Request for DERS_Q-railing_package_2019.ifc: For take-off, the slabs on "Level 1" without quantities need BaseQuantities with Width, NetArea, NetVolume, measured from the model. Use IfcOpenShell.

First a look at what the model holds.

```python
import ifcopenshell
import ifcopenshell.util.element
import ifcopenshell.util.unit

model = ifcopenshell.open("DERS_Q-railing_package_2019.ifc")
print(model.schema)
for unit_type in ("LENGTHUNIT", "AREAUNIT", "VOLUMEUNIT"):
    print(unit_type, ifcopenshell.util.unit.calculate_unit_scale(model, unit_type))
storey = next(s for s in model.by_type("IfcBuildingStorey") if s.Name == "Level 1")
slabs = [e for e in ifcopenshell.util.element.get_decomposition(storey) if e.is_a("IfcSlab")]
for e in sorted(slabs, key=lambda e: e.id()):
    print(e.id(), e.is_a(), e.Name, list(ifcopenshell.util.element.get_psets(e, qtos_only=True)), sep=" | ")
```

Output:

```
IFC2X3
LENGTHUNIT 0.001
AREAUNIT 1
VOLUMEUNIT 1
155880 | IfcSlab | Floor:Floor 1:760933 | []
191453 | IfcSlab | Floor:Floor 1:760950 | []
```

```python
import ifcopenshell
import ifcopenshell.api.pset
import ifcopenshell.geom
import ifcopenshell.util.element
import ifcopenshell.util.shape
import ifcopenshell.util.unit

model = ifcopenshell.open("DERS_Q-railing_package_2019.ifc")
unit_scale = ifcopenshell.util.unit.calculate_unit_scale(model)
area_scale = ifcopenshell.util.unit.calculate_unit_scale(model, "AREAUNIT")
volume_scale = ifcopenshell.util.unit.calculate_unit_scale(model, "VOLUMEUNIT")
settings = ifcopenshell.geom.settings()

storey = next(s for s in model.by_type("IfcBuildingStorey") if s.Name == "Level 1")
slabs = [e for e in ifcopenshell.util.element.get_decomposition(storey) if e.is_a("IfcSlab")]

for e in sorted(slabs, key=lambda e: e.id()):
    if ifcopenshell.util.element.get_psets(e, qtos_only=True, should_inherit=False):
        continue
    # Geometry comes back in metres, in the element's own axes.
    shape = ifcopenshell.geom.create_shape(settings, e)
    values = {
        "Width": ifcopenshell.util.shape.get_z(shape.geometry) / unit_scale,
        "NetArea": ifcopenshell.util.shape.get_footprint_area(shape.geometry) / area_scale,
        "NetVolume": ifcopenshell.util.shape.get_volume(shape.geometry) / volume_scale,
    }
    qto = ifcopenshell.api.pset.add_qto(model, product=e, name="BaseQuantities")
    ifcopenshell.api.pset.edit_qto(model, qto=qto, properties=values)
    print(e.id(), {k: round(v, 3) for k, v in values.items()})

model.write("DERS_Q-railing_package_2019-out.ifc")
```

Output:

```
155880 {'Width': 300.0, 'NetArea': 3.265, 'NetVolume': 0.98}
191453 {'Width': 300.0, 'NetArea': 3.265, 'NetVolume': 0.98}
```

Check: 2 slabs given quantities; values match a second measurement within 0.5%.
